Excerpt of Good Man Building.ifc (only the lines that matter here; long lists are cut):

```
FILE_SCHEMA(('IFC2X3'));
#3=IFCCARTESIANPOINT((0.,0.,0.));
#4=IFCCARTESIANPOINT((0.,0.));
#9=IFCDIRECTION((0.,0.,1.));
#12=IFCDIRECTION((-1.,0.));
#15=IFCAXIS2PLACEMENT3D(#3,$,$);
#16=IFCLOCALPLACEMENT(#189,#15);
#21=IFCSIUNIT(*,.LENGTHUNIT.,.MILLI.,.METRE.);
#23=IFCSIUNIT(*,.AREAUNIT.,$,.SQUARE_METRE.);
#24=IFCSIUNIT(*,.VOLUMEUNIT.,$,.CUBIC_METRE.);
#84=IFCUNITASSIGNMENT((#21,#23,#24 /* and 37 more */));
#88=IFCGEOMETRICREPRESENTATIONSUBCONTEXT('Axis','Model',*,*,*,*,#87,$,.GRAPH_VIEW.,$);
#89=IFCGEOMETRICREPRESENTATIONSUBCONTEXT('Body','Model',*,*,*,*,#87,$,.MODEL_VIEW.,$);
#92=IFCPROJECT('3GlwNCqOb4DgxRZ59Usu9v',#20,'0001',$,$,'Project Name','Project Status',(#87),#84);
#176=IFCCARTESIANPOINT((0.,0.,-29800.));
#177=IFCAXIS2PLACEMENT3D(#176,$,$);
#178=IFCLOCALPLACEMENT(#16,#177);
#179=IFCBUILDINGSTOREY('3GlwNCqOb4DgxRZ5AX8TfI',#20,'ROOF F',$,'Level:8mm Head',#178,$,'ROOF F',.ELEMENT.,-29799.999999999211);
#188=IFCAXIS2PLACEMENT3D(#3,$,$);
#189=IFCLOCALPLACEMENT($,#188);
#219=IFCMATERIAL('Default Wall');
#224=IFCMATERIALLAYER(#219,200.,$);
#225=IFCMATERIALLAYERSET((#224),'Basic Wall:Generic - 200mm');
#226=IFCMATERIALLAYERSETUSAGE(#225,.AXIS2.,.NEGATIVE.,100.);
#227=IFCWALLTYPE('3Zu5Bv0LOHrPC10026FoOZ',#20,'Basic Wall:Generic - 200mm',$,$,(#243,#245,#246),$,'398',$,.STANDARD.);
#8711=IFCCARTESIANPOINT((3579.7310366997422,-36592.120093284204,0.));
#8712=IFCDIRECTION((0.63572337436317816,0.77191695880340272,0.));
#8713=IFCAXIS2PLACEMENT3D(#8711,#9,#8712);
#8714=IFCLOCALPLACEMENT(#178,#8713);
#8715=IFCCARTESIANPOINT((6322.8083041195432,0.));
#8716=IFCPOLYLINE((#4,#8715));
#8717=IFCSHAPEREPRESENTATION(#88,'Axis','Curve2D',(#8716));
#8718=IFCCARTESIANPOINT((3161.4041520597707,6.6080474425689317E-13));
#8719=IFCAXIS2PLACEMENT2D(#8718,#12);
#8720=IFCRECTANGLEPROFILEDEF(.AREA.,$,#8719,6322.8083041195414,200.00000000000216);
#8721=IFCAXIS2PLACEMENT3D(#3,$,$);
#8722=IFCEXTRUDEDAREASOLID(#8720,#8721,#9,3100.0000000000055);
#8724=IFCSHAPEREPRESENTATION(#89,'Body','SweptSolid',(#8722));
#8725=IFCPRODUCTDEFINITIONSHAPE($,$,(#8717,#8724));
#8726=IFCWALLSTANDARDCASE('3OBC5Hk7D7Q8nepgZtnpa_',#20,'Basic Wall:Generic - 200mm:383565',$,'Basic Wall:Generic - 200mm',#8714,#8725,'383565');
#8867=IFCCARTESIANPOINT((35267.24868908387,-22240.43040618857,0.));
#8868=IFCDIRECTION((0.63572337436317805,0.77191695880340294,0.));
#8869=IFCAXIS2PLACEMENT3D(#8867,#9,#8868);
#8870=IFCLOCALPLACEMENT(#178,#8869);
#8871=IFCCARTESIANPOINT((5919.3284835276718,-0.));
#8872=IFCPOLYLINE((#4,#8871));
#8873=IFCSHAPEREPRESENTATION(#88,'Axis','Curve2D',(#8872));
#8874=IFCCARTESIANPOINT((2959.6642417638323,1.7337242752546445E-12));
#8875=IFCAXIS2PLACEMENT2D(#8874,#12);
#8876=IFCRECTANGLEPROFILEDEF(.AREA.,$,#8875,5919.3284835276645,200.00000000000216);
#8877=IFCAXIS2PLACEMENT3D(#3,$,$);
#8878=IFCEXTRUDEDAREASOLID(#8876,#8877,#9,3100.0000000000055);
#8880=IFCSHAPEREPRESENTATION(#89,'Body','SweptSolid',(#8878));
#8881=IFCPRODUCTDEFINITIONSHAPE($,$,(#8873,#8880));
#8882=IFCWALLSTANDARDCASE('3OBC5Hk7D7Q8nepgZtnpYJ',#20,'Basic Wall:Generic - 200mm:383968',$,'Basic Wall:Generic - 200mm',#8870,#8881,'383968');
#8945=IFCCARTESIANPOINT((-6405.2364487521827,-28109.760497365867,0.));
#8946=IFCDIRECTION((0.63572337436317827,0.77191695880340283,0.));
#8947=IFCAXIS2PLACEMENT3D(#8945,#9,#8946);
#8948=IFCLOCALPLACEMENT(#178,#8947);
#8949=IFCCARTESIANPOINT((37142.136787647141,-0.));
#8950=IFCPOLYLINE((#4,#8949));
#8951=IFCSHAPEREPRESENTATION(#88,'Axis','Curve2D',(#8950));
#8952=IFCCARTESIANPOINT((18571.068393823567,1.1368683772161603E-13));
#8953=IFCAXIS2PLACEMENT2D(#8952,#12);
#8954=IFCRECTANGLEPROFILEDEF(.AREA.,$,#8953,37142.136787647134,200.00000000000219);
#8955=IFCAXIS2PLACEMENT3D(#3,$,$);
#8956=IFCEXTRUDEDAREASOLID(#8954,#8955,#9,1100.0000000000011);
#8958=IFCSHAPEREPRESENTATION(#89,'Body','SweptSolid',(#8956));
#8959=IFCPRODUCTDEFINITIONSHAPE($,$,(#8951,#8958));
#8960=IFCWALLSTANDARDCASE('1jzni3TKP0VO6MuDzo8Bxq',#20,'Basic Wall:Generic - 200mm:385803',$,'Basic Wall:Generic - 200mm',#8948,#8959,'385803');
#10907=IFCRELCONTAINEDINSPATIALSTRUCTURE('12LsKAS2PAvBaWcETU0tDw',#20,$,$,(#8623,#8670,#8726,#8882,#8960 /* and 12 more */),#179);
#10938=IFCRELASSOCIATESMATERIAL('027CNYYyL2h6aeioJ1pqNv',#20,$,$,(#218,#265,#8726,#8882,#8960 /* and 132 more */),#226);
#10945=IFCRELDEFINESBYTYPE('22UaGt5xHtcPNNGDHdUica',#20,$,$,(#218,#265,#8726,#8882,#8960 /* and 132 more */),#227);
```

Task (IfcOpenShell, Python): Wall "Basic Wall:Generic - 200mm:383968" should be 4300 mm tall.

```python
import ifcopenshell
import ifcopenshell.geom
import ifcopenshell.util.representation
import ifcopenshell.util.shape
import ifcopenshell.util.unit

model = ifcopenshell.open("Good Man Building.ifc")
unit_scale = ifcopenshell.util.unit.calculate_unit_scale(model)
settings = ifcopenshell.geom.settings()


def volume(element):
    """Net volume in cubic metres, openings subtracted."""
    shape = ifcopenshell.geom.create_shape(settings, element)
    return ifcopenshell.util.shape.get_volume(shape.geometry)


wall = model.by_id(8882)
before = volume(wall)

body = ifcopenshell.util.representation.get_representation(wall, "Model", "Body")
solid = body.Items[0]
old_height = solid.Depth
solid.Depth = 4.3 / unit_scale
after = volume(wall)

print(f"height {old_height:g} -> {solid.Depth:g}, volume {before:.3f} -> {after:.3f} m3")

model.write("Good Man Building-out.ifc")
```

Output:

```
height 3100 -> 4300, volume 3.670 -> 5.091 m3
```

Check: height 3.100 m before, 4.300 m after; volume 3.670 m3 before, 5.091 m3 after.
